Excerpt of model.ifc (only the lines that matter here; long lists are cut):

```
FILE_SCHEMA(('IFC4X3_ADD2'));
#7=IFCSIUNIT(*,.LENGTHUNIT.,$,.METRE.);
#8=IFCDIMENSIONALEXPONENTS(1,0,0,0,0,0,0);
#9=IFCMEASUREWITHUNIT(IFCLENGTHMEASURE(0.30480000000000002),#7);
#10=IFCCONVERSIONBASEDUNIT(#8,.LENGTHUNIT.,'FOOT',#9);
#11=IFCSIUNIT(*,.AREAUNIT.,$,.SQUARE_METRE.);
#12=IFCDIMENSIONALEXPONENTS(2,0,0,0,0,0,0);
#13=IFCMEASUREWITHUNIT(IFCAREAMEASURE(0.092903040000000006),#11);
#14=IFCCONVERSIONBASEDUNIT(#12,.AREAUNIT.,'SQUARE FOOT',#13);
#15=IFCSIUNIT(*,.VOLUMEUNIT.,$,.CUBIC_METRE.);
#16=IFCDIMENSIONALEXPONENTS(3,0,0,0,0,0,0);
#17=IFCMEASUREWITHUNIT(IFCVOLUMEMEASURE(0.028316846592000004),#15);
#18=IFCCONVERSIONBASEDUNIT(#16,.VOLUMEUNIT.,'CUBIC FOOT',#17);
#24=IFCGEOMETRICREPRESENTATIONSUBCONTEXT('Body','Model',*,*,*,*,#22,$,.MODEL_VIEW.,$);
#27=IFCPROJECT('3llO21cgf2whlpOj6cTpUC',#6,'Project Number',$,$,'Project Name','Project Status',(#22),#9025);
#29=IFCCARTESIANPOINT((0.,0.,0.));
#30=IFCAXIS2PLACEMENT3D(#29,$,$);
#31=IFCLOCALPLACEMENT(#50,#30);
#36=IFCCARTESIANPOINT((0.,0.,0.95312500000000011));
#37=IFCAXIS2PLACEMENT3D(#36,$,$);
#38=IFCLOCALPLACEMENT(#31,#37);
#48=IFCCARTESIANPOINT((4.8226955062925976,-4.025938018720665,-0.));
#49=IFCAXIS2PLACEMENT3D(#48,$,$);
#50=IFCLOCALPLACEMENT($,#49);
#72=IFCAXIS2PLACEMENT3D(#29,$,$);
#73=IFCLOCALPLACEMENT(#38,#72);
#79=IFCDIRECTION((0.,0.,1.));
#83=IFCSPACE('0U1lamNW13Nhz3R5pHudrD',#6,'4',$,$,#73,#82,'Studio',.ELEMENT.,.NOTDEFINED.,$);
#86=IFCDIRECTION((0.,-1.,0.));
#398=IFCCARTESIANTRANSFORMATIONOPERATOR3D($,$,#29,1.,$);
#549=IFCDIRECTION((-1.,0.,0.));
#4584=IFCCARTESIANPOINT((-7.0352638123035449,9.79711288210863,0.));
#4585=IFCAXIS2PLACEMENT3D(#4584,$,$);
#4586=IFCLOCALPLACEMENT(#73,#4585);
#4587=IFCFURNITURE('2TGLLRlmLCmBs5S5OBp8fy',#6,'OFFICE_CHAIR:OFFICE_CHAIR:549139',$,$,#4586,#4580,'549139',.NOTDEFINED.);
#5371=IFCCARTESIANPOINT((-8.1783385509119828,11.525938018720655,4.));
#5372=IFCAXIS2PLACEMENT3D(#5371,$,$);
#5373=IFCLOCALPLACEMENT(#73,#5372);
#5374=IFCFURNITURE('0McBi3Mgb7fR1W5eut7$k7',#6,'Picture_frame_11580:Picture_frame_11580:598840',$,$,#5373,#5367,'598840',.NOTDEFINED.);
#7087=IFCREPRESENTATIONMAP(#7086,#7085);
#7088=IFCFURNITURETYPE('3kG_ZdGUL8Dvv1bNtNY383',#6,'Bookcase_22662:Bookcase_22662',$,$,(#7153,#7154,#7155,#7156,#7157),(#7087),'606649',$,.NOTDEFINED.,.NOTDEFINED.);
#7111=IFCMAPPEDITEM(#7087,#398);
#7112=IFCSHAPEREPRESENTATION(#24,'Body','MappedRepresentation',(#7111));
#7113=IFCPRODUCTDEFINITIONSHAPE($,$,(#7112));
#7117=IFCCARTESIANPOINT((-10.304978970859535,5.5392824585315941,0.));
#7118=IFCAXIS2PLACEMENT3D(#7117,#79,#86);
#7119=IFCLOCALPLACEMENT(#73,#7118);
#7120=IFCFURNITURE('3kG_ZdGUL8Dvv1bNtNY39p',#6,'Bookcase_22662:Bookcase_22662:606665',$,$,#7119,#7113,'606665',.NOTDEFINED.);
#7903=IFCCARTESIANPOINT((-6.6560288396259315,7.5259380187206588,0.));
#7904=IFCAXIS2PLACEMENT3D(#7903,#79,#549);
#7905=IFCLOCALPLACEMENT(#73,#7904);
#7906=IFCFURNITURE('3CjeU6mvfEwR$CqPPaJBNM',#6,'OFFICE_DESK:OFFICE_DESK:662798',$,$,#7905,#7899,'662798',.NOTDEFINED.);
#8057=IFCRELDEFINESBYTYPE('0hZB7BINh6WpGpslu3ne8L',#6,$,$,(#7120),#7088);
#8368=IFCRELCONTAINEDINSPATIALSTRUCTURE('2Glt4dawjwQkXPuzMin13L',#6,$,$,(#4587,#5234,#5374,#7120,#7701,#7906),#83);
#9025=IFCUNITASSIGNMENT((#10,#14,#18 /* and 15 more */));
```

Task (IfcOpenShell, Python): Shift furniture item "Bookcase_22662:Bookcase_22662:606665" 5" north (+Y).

```python
import ifcopenshell
import ifcopenshell.api.geometry
import ifcopenshell.util.placement
import ifcopenshell.util.unit

model = ifcopenshell.open("model.ifc")
unit_scale = ifcopenshell.util.unit.calculate_unit_scale(model)

item = model.by_guid("3kG_ZdGUL8Dvv1bNtNY39p")
matrix = ifcopenshell.util.placement.get_local_placement(item.ObjectPlacement)
matrix[1, 3] += 5 * 0.0254 / unit_scale
ifcopenshell.api.geometry.edit_object_placement(model, product=item, matrix=matrix, is_si=False)

print(ifcopenshell.util.placement.get_local_placement(item.ObjectPlacement).round(3) + 0.0)

model.write("model_v2.ifc")
```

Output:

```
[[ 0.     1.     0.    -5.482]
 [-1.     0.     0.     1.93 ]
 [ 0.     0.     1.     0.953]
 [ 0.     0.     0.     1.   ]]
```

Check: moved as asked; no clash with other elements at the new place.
